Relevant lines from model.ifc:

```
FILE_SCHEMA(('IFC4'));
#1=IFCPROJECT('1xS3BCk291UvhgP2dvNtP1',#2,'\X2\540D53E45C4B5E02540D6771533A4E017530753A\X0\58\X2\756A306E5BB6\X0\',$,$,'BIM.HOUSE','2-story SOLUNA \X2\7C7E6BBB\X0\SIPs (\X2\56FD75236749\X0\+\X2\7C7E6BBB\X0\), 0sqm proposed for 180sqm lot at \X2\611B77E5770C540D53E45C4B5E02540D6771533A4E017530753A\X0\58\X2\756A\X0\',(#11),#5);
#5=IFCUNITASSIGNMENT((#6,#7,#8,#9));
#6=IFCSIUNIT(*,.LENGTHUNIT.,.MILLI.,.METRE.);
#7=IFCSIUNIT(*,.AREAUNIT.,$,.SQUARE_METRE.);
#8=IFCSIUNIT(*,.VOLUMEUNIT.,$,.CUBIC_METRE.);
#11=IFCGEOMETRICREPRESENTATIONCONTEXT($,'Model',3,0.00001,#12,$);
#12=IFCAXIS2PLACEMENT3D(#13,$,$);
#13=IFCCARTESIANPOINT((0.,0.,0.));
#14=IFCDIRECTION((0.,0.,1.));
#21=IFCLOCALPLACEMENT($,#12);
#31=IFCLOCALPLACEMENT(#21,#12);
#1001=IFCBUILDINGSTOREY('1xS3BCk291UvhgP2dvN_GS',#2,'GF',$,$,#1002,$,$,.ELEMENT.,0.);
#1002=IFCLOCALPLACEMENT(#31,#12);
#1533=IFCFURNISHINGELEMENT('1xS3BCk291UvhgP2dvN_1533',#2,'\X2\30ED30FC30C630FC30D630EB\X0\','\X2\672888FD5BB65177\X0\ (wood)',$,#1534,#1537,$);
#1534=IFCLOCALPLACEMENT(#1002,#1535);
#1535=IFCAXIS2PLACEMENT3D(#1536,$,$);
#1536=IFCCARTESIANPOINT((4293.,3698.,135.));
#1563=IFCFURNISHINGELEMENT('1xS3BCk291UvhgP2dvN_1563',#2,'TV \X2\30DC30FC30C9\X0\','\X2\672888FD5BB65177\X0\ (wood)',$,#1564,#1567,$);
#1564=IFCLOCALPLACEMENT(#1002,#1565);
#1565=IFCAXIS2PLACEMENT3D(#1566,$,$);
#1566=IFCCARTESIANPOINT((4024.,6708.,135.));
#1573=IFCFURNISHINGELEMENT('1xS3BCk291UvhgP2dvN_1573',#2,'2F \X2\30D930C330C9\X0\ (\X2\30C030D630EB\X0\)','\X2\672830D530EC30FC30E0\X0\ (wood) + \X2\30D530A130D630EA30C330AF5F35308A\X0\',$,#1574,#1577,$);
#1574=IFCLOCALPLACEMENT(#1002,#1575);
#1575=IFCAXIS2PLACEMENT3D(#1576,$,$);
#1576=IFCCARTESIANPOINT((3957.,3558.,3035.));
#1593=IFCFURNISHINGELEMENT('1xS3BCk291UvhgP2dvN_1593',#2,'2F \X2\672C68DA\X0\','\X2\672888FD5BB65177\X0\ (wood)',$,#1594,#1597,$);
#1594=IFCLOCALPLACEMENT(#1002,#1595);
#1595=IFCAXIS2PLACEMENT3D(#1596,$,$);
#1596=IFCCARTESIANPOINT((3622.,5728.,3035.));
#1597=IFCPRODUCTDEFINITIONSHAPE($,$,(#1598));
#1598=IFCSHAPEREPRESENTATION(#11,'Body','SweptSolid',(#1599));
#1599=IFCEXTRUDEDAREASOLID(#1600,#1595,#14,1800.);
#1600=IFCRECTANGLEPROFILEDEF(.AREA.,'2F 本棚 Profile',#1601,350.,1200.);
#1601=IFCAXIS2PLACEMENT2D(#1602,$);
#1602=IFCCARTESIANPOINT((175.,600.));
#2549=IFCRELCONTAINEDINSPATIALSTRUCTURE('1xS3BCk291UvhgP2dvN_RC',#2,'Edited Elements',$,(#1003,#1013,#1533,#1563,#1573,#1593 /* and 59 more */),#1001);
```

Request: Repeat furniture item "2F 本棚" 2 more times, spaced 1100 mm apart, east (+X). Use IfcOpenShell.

```python
import numpy as np
import ifcopenshell
import ifcopenshell.api.geometry
import ifcopenshell.api.root
import ifcopenshell.util.element
import ifcopenshell.util.placement

model = ifcopenshell.open("model.ifc")


def reuse_history(source, copy):
    """copy_class also copies each property set's owner history, people and application; keep the originals."""
    for rel in copy.IsDefinedBy:
        if rel.is_a("IfcRelDefinesByProperties") and (history := rel.RelatingPropertyDefinition.OwnerHistory):
            rel.RelatingPropertyDefinition.OwnerHistory = source.OwnerHistory
            ifcopenshell.util.element.remove_deep2(model, history)


source = model.by_guid("1xS3BCk291UvhgP2dvN_1593")
base = ifcopenshell.util.placement.get_local_placement(source.ObjectPlacement)
step = np.array([1.0, 0.0, 0.0]) * 1100.0

for i in range(1, 3):
    copy = ifcopenshell.api.root.copy_class(model, product=source)
    copy.Representation = ifcopenshell.util.element.copy_deep(
        model, source.Representation, exclude=["IfcGeometricRepresentationContext", "IfcRepresentationMap"]
    )
    reuse_history(source, copy)
    matrix = base.copy()
    matrix[:3, 3] += i * step
    print("added at", matrix[:3, 3].round(3) + 0.0)
    ifcopenshell.api.geometry.edit_object_placement(model, product=copy, matrix=matrix, is_si=False)

model.write("model_edited.ifc")
```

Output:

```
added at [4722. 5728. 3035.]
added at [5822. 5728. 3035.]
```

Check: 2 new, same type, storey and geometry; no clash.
